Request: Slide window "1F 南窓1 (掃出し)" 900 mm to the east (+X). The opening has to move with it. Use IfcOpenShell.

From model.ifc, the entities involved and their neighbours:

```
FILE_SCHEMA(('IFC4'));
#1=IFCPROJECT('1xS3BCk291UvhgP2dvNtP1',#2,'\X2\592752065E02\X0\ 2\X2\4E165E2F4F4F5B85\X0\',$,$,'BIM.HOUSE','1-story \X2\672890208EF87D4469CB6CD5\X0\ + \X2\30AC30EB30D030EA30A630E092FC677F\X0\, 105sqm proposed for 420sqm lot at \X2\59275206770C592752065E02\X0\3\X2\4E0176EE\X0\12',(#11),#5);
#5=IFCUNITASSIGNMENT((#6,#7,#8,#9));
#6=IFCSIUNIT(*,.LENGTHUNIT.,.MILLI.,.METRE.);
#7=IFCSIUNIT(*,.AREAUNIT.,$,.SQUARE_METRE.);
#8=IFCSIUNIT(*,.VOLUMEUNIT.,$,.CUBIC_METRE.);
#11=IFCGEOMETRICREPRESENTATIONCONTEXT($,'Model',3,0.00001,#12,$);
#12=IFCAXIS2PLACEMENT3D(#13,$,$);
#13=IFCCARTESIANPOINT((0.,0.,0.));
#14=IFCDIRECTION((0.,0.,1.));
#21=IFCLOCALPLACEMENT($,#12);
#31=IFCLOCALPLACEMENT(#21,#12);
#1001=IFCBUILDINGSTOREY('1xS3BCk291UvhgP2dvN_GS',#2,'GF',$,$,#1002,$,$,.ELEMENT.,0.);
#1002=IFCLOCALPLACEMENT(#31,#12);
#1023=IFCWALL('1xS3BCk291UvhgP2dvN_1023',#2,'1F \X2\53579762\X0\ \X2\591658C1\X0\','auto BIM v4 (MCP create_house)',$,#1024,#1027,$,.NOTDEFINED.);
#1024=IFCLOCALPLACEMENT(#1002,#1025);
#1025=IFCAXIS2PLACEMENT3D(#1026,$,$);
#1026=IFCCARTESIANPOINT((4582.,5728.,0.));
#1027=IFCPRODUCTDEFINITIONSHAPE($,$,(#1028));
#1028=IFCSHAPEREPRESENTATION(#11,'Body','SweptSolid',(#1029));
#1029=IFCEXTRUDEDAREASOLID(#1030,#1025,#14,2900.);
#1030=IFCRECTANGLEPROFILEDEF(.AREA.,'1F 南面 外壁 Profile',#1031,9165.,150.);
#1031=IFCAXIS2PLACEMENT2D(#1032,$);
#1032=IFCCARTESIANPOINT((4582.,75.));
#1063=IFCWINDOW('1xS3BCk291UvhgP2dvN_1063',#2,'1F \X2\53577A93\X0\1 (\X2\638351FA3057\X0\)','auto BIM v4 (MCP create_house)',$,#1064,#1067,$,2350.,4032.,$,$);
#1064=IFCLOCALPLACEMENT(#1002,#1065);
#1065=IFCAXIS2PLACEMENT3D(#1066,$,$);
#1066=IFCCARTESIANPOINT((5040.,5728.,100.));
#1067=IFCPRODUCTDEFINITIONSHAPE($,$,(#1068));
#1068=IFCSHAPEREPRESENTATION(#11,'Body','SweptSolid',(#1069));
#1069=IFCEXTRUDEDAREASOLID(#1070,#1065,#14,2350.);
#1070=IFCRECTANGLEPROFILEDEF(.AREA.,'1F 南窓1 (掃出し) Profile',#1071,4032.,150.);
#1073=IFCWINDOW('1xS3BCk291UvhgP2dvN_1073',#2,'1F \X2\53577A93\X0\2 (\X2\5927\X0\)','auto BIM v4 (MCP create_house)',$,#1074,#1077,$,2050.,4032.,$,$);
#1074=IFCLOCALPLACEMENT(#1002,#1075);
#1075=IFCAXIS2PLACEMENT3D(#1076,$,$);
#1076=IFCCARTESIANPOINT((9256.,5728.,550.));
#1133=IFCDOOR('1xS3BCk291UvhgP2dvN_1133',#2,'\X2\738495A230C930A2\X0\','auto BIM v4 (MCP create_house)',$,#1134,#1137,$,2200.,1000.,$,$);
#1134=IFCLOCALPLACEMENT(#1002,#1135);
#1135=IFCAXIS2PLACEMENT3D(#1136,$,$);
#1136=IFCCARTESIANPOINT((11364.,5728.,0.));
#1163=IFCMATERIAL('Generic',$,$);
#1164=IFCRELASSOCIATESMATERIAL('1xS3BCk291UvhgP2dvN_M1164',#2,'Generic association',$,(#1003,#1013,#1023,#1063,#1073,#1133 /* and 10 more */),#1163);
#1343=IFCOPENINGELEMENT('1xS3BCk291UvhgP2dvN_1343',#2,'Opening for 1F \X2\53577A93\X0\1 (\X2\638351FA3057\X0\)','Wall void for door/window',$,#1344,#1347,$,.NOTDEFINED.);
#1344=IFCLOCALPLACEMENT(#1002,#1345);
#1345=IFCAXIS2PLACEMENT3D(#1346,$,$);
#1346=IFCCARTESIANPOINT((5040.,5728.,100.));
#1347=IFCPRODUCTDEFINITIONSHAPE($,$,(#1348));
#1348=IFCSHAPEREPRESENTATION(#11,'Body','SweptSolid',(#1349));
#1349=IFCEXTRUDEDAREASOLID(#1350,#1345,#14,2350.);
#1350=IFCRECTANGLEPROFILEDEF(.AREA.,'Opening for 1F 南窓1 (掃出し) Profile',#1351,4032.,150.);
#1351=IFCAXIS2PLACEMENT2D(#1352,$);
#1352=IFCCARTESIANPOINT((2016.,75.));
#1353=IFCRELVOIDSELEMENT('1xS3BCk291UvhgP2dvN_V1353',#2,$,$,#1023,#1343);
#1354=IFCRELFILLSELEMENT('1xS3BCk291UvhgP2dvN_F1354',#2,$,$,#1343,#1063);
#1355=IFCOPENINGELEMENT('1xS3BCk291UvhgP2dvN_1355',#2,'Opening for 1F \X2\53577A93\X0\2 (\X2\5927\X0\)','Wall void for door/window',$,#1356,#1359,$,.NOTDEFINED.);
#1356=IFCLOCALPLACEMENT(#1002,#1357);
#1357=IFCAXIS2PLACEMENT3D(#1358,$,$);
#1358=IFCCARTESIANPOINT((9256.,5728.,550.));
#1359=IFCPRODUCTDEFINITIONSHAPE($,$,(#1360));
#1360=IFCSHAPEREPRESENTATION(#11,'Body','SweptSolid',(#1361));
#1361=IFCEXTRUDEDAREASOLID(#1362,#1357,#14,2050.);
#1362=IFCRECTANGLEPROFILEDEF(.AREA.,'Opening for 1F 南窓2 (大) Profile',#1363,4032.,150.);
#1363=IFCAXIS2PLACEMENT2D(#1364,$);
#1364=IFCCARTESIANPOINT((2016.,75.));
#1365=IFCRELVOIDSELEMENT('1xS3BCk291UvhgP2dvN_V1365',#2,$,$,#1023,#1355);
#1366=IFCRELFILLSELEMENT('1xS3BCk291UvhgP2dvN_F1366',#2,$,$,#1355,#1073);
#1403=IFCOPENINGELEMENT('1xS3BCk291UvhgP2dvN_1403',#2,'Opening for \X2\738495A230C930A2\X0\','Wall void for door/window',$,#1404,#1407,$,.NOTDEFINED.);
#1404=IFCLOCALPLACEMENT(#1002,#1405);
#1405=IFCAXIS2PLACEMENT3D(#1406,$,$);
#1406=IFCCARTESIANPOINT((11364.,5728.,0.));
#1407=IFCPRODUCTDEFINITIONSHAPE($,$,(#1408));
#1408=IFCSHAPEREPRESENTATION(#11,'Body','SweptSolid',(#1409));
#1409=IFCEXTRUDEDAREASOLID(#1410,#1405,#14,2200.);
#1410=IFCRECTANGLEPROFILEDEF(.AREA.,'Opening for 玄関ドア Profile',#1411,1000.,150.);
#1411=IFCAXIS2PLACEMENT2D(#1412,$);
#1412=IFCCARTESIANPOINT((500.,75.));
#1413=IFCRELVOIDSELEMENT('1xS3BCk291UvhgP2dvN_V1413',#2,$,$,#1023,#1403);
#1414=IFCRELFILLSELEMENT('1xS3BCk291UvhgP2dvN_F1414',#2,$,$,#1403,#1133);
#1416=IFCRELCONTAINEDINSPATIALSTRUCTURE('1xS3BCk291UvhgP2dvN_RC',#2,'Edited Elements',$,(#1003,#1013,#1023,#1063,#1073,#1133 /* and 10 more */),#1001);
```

```python
import ifcopenshell
import ifcopenshell.api.geometry
import ifcopenshell.util.placement
import ifcopenshell.util.unit

model = ifcopenshell.open("model.ifc")
unit_scale = ifcopenshell.util.unit.calculate_unit_scale(model)

window = model.by_id(1063)
opening = window.FillsVoids[0].RelatingOpeningElement
wall = opening.VoidsElements[0].RelatingBuildingElement

wall_matrix = ifcopenshell.util.placement.get_local_placement(wall.ObjectPlacement)
shift = wall_matrix[:3, 0] * 0.9 / unit_scale
before = ifcopenshell.util.placement.get_local_placement(window.ObjectPlacement)[:3, 3].copy()

# The window is not placed relative to its opening, so move both.
for product in (opening, window):
    matrix = ifcopenshell.util.placement.get_local_placement(product.ObjectPlacement)
    matrix[:3, 3] += shift
    ifcopenshell.api.geometry.edit_object_placement(model, product=product, matrix=matrix, is_si=False)

after = ifcopenshell.util.placement.get_local_placement(window.ObjectPlacement)[:3, 3]
print("window moved by", (after - before).round(3) + 0.0)

model.write("model_updated.ifc")
```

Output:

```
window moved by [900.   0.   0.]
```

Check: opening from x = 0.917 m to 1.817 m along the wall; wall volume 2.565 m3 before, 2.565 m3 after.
